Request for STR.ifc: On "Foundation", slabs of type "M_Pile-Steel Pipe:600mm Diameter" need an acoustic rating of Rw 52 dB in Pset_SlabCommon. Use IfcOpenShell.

First a look at what the model holds.

```python
import ifcopenshell
import ifcopenshell.util.element

model = ifcopenshell.open("STR.ifc")
print(model.schema)
storey = next(s for s in model.by_type("IfcBuildingStorey") if s.Name == "Foundation")
slabs = [e for e in ifcopenshell.util.element.get_decomposition(storey) if e.is_a("IfcSlab")]
seen = {}
for e in slabs:
    element_type = ifcopenshell.util.element.get_type(e)
    key = (element_type.Name if element_type != e and element_type else None, ifcopenshell.util.element.get_pset(e, "Pset_SlabCommon", "AcousticRating"))
    seen[key] = seen.get(key, 0) + 1
for (name, value), count in sorted(seen.items(), key=str):
    print(count, "x", name, "|", value)
```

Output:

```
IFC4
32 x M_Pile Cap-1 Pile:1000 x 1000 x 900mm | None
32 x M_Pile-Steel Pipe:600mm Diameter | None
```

```python
import ifcopenshell
import ifcopenshell.api.pset
import ifcopenshell.util.element

model = ifcopenshell.open("STR.ifc")

storey = next(s for s in model.by_type("IfcBuildingStorey") if s.Name == "Foundation")
slabs = [e for e in ifcopenshell.util.element.get_decomposition(storey) if e.is_a("IfcSlab")]

count = 0
for e in slabs:
    element_type = ifcopenshell.util.element.get_type(e)
    if element_type in (None, e) or element_type.Name != "M_Pile-Steel Pipe:600mm Diameter":
        continue
    # add_pset returns the element's existing set when there is one.
    pset = ifcopenshell.api.pset.add_pset(model, product=e, name="Pset_SlabCommon")
    ifcopenshell.api.pset.edit_pset(model, pset=pset, properties={"AcousticRating": "Rw 52 dB"})
    count += 1

print(count, "slabs updated")

model.write("STR_edited.ifc")
```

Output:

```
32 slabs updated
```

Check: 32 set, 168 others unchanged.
